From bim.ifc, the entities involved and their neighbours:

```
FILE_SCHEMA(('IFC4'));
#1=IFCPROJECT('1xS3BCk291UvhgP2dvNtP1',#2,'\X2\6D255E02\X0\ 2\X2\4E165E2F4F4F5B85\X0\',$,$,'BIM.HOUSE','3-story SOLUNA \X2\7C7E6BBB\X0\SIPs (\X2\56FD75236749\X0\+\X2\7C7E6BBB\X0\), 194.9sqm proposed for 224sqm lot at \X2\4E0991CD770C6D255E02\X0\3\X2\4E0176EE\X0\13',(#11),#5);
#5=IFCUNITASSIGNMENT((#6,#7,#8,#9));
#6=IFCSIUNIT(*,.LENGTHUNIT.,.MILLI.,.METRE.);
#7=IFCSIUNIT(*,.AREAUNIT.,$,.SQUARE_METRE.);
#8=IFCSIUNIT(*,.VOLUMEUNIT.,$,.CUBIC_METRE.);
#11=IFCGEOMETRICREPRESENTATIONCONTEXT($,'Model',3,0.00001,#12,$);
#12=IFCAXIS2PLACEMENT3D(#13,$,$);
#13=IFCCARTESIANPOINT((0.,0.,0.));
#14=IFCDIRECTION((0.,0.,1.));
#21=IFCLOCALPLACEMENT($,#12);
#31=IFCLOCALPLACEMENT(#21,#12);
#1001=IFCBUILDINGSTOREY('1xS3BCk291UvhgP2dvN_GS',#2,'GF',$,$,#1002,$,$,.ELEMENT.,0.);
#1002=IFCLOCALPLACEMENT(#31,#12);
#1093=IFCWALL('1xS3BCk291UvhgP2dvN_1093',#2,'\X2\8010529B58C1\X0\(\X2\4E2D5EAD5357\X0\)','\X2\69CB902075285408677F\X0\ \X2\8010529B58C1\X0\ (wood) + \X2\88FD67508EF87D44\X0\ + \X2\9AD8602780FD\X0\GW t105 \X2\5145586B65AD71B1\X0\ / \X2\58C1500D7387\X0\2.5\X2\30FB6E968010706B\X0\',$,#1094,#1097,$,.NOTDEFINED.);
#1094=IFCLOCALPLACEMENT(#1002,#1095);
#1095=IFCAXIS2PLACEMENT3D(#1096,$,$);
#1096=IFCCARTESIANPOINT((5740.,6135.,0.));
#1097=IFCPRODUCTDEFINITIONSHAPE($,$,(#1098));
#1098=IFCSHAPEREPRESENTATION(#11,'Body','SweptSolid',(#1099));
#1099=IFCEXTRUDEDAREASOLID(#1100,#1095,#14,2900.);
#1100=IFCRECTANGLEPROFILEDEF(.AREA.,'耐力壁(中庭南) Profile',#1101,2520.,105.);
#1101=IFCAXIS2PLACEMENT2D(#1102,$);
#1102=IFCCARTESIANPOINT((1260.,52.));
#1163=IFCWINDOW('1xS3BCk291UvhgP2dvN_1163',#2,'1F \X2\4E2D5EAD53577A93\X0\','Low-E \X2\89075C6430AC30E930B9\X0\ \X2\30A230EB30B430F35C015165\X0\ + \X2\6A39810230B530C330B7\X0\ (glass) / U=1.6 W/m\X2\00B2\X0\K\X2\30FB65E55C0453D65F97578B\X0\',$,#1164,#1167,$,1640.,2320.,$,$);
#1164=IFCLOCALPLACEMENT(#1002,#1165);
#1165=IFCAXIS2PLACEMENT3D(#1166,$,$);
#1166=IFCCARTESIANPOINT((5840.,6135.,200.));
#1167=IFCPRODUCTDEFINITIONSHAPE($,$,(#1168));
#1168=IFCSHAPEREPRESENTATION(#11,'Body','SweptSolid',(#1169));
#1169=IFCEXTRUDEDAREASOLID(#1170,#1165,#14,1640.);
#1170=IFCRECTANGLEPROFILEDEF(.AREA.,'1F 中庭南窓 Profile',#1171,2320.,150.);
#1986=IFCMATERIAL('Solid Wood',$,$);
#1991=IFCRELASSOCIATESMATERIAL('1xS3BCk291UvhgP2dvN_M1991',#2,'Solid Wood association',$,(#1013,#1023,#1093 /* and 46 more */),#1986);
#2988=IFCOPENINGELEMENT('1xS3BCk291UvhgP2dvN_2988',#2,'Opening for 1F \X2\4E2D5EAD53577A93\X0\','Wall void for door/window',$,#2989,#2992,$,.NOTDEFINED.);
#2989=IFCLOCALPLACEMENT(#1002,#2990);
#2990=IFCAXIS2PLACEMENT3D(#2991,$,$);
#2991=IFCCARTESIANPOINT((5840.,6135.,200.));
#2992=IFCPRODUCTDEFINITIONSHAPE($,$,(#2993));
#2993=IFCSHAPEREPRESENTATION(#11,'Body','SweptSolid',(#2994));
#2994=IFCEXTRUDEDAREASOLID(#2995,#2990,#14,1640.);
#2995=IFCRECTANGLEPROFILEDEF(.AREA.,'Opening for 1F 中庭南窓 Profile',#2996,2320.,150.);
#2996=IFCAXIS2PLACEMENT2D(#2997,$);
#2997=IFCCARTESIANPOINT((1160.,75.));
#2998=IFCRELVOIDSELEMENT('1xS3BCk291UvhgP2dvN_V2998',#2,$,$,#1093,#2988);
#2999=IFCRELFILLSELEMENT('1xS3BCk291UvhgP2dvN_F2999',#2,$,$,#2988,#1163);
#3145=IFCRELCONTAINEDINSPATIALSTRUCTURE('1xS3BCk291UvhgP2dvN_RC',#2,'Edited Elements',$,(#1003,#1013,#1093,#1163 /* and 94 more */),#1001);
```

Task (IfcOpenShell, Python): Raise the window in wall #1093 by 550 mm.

```python
import numpy as np
import ifcopenshell
import ifcopenshell.api.geometry
import ifcopenshell.util.placement
import ifcopenshell.util.unit

model = ifcopenshell.open("bim.ifc")
unit_scale = ifcopenshell.util.unit.calculate_unit_scale(model)

window = model.by_id(1163)
opening = window.FillsVoids[0].RelatingOpeningElement
dz = 550.0

shift = np.array([0.0, 0.0, dz])
# The window is not placed relative to its opening, so move both.
for product in (opening, window):
    matrix = ifcopenshell.util.placement.get_local_placement(product.ObjectPlacement)
    matrix[:3, 3] += shift
    ifcopenshell.api.geometry.edit_object_placement(model, product=product, matrix=matrix, is_si=False)

print(f"moved by {dz * unit_scale:+.3f} m")

model.write("bim_edited.ifc")
```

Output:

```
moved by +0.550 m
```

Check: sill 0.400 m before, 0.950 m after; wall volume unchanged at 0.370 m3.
